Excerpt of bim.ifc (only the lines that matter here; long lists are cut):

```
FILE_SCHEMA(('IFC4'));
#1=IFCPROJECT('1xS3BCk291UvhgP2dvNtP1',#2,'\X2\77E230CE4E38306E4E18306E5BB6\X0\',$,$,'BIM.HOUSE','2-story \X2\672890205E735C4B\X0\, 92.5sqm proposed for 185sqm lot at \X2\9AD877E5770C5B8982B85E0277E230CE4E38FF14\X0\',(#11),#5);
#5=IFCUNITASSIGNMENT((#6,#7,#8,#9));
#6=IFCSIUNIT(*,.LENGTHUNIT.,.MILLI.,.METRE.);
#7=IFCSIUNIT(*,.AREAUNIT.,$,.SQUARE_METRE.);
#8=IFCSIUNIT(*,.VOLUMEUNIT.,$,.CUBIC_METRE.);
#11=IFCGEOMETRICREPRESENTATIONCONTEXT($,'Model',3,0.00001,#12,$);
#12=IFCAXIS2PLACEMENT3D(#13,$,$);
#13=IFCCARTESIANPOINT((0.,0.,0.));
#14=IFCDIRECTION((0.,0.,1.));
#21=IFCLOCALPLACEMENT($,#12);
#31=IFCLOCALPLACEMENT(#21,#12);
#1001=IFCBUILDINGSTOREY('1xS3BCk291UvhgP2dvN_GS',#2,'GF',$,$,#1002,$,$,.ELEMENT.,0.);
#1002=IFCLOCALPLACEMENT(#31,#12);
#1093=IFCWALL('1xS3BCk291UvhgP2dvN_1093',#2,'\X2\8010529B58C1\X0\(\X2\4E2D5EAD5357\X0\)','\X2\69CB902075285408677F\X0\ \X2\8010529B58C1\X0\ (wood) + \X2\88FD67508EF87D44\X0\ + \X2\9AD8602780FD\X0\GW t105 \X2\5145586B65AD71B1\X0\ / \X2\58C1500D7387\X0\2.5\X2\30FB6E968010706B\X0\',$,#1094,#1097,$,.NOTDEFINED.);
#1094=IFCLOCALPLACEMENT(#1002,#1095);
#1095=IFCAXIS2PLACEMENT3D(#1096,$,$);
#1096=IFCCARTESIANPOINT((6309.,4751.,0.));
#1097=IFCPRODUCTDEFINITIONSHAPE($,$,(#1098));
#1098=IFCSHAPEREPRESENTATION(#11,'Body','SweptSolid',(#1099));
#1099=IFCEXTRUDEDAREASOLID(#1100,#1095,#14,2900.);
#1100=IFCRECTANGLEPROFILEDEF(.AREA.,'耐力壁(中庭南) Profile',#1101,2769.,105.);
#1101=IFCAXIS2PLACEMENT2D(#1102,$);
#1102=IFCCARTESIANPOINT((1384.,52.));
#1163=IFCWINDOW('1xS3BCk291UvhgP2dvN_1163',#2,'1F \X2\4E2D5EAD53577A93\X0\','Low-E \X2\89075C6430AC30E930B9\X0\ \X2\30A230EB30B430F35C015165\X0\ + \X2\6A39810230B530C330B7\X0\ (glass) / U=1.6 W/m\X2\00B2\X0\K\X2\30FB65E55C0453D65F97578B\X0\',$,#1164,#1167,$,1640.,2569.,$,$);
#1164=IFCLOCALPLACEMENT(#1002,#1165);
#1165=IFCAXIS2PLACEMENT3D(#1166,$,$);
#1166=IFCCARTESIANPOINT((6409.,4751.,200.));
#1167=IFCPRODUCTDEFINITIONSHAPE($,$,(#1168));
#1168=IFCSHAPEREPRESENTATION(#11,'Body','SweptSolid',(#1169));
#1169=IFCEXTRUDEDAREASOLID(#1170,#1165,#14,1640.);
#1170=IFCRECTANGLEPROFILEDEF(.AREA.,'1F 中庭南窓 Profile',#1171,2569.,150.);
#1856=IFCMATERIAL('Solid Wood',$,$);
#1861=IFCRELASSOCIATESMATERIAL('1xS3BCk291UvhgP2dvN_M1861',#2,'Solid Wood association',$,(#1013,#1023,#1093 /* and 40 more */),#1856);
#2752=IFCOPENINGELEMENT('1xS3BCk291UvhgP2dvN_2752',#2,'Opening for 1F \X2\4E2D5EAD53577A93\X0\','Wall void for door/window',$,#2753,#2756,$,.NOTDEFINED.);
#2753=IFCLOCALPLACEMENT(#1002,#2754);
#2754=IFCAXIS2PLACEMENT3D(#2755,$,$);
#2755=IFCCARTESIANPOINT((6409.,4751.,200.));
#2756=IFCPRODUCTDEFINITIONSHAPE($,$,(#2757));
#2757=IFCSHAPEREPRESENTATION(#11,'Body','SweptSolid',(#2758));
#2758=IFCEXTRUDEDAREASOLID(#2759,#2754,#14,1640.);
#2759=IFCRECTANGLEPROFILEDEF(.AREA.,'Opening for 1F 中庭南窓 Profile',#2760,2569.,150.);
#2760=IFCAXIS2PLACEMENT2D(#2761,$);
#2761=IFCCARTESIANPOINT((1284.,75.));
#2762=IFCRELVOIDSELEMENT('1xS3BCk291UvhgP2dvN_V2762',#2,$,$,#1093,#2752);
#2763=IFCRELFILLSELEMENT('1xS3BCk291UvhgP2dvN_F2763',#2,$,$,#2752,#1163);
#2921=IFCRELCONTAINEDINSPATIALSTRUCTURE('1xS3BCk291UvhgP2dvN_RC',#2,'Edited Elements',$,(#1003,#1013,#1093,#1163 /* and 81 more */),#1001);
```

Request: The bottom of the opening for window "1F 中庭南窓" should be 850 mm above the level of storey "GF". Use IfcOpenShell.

```python
import numpy as np
import ifcopenshell
import ifcopenshell.api.geometry
import ifcopenshell.geom
import ifcopenshell.util.element
import ifcopenshell.util.placement
import ifcopenshell.util.shape
import ifcopenshell.util.unit

model = ifcopenshell.open("bim.ifc")
unit_scale = ifcopenshell.util.unit.calculate_unit_scale(model)

window = model.by_id(1163)
opening = window.FillsVoids[0].RelatingOpeningElement
storey = ifcopenshell.util.element.get_container(window, ifc_class="IfcBuildingStorey")
level = ifcopenshell.util.placement.get_local_placement(storey.ObjectPlacement)[2, 3]

# The opening's origin need not be at the sill, so measure its lowest point.
shape = ifcopenshell.geom.create_shape(ifcopenshell.geom.settings(), opening)
bottom = ifcopenshell.util.shape.get_shape_bottom_elevation(shape, shape.geometry) / unit_scale
dz = level + 0.85 / unit_scale - bottom

shift = np.array([0.0, 0.0, dz])
# The window is not placed relative to its opening, so move both.
for product in (opening, window):
    matrix = ifcopenshell.util.placement.get_local_placement(product.ObjectPlacement)
    matrix[:3, 3] += shift
    ifcopenshell.api.geometry.edit_object_placement(model, product=product, matrix=matrix, is_si=False)

print(f"moved by {dz * unit_scale:+.3f} m")

model.write("bim-out.ifc")
```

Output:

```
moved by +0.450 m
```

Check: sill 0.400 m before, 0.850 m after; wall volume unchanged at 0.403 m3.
